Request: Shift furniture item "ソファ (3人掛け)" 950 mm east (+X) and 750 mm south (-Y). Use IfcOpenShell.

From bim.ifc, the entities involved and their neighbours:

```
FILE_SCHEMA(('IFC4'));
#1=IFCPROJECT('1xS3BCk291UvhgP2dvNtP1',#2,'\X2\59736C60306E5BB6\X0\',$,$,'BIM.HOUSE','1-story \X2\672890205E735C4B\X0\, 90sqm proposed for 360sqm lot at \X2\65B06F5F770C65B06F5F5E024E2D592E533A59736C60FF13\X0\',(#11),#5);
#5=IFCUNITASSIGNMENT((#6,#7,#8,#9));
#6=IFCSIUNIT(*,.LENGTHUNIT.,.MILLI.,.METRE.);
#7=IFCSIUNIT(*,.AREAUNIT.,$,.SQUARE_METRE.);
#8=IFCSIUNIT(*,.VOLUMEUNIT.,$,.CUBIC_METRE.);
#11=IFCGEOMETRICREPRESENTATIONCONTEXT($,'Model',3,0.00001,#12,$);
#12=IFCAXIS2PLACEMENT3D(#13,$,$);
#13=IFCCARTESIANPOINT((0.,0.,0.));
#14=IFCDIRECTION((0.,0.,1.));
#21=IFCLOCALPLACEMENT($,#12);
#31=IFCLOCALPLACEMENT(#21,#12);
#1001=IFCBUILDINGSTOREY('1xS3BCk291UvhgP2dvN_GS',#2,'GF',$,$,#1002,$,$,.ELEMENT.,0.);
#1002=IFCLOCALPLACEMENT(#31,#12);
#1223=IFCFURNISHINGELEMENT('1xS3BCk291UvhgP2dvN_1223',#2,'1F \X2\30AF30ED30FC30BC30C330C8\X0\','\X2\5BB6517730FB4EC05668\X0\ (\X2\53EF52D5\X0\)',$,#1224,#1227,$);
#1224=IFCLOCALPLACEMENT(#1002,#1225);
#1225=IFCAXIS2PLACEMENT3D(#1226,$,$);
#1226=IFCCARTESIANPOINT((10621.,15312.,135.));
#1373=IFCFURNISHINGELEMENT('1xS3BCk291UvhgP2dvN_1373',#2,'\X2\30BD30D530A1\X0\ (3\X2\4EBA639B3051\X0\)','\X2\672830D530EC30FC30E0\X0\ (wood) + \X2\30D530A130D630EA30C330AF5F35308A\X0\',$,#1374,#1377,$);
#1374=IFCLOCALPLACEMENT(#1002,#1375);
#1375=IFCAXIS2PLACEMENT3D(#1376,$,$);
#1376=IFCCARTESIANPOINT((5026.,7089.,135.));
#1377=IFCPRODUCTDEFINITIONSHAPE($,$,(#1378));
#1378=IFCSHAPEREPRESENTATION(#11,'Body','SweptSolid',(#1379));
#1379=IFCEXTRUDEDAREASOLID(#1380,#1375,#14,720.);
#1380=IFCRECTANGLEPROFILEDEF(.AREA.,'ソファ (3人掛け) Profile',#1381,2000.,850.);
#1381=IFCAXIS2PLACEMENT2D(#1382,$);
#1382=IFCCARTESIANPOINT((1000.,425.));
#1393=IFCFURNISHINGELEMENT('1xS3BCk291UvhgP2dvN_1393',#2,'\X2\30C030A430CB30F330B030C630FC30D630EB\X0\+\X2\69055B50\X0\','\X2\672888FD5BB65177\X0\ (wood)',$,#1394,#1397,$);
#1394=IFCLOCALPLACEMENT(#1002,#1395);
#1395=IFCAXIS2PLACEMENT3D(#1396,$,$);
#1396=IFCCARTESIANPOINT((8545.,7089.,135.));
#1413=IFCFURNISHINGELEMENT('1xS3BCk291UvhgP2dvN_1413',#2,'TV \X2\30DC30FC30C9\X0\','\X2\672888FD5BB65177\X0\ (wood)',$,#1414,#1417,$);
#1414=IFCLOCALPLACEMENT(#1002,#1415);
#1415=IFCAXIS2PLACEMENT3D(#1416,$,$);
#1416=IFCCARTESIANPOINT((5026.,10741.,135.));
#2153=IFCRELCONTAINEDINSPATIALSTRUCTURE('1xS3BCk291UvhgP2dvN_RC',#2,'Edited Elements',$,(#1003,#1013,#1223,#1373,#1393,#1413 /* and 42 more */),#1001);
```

```python
import ifcopenshell
import ifcopenshell.api.geometry
import ifcopenshell.util.placement
import ifcopenshell.util.unit

model = ifcopenshell.open("bim.ifc")
unit_scale = ifcopenshell.util.unit.calculate_unit_scale(model)

item = model.by_id(1373)
matrix = ifcopenshell.util.placement.get_local_placement(item.ObjectPlacement)
matrix[0, 3] += 0.95 / unit_scale
matrix[1, 3] -= 0.75 / unit_scale
ifcopenshell.api.geometry.edit_object_placement(model, product=item, matrix=matrix, is_si=False)

print(ifcopenshell.util.placement.get_local_placement(item.ObjectPlacement).round(3) + 0.0)

model.write("bim_edited.ifc")
```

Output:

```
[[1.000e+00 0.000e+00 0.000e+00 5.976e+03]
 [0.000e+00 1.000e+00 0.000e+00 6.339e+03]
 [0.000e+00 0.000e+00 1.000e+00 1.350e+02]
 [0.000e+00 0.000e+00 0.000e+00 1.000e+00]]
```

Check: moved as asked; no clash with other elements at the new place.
